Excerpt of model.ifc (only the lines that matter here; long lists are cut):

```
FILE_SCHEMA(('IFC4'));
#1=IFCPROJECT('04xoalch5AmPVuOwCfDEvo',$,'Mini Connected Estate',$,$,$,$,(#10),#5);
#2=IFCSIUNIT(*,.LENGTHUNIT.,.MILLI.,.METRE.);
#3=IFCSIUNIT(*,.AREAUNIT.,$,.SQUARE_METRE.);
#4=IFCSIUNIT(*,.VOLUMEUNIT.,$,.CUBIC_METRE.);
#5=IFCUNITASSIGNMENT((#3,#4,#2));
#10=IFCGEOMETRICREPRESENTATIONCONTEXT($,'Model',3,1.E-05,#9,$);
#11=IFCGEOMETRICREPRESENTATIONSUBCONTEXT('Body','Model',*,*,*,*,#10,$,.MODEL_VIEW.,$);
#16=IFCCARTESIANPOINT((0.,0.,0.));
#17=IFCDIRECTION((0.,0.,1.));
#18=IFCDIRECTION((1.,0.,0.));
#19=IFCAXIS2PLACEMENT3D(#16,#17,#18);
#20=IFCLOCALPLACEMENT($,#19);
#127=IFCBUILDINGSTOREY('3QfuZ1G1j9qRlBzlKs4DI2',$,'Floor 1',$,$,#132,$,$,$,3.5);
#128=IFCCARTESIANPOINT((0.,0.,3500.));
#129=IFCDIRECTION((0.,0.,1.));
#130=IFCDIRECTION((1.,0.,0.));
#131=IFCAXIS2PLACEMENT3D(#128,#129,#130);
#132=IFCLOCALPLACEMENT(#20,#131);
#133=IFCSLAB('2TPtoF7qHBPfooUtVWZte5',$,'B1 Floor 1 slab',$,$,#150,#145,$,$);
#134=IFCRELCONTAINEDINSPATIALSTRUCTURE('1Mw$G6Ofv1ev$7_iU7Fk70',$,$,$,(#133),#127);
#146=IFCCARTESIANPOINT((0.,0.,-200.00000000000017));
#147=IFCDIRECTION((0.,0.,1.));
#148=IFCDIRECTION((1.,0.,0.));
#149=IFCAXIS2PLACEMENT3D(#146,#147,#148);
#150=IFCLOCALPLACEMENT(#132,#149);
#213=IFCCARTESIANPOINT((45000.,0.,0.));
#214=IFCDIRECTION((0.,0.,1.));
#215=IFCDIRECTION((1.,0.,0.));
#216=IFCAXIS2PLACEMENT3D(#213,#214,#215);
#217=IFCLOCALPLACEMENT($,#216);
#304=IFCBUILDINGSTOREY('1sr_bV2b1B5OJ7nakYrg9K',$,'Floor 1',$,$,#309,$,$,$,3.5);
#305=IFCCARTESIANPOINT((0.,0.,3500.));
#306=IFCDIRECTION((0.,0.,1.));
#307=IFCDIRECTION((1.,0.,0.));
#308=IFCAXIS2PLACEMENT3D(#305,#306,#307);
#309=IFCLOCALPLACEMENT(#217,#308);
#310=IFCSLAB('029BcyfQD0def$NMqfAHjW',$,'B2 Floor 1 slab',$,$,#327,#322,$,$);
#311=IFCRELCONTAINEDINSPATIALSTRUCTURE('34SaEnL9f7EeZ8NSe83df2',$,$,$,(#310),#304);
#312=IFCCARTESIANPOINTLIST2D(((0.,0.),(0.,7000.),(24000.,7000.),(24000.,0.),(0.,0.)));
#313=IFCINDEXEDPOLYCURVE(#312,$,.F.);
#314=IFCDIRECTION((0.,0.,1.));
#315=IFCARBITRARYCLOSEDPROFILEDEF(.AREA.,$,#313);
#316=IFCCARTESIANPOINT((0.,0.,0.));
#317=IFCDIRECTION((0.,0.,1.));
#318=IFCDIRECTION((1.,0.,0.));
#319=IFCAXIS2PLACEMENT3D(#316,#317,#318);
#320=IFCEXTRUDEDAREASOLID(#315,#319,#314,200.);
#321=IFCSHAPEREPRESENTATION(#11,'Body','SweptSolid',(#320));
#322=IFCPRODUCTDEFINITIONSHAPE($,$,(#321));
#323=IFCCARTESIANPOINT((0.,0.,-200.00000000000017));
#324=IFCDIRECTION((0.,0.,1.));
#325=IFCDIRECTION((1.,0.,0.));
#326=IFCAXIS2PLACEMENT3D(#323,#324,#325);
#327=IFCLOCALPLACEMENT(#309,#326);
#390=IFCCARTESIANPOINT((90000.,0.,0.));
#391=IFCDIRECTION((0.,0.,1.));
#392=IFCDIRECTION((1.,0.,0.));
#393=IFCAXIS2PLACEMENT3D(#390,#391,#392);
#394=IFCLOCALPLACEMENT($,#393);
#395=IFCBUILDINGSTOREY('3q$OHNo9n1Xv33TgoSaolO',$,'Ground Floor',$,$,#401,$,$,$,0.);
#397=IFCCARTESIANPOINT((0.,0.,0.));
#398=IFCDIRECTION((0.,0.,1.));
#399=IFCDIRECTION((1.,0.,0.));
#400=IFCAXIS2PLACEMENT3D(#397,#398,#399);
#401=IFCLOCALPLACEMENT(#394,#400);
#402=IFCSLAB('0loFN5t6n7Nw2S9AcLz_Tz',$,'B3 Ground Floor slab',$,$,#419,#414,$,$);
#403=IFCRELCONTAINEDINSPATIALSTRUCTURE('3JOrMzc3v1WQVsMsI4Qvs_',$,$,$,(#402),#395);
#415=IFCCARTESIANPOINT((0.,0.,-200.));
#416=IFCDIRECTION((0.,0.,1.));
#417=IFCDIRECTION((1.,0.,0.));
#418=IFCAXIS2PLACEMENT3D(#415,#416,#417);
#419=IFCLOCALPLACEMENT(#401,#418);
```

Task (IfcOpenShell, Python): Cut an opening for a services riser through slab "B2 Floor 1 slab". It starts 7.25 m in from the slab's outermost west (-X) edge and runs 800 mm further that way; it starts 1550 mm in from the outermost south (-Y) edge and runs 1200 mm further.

```python
import numpy as np
import ifcopenshell
import ifcopenshell.api.feature
import ifcopenshell.api.geometry
import ifcopenshell.api.root
import ifcopenshell.geom
import ifcopenshell.util.placement
import ifcopenshell.util.representation
import ifcopenshell.util.shape
import ifcopenshell.util.unit

model = ifcopenshell.open("model.ifc")
unit_scale = ifcopenshell.util.unit.calculate_unit_scale(model)
settings = ifcopenshell.geom.settings()


def volume(element):
    """Net volume in cubic metres, openings subtracted."""
    shape = ifcopenshell.geom.create_shape(settings, element)
    return ifcopenshell.util.shape.get_volume(shape.geometry)


slab = model.by_id(310)
before = volume(slab)

# Extent in the slab's own axes, in metres. The edges named are its -X and -Y sides.
slab_shape = ifcopenshell.geom.create_shape(settings, slab)
vertices = ifcopenshell.util.shape.get_vertices(slab_shape.geometry)
x_min, y_min, bottom = vertices.min(axis=0)
top = vertices[:, 2].max()

opening = ifcopenshell.api.root.create_entity(model, ifc_class="IfcOpeningElement", name="Services riser opening", predefined_type="OPENING")
context = ifcopenshell.util.representation.get_context(model, "Model", "Body", "MODEL_VIEW")
width, depth = 0.8, 1.2
outline = [(0.0, 0.0), (width, 0.0), (width, depth), (0.0, depth), (0.0, 0.0)]
# Overshoot both faces by 50 mm so the cut is clean.
shape = ifcopenshell.api.geometry.add_slab_representation(
    model, context=context, depth=top - bottom + 0.1, polyline=outline
)
ifcopenshell.api.geometry.assign_representation(model, product=opening, representation=shape)

matrix = ifcopenshell.util.placement.get_local_placement(slab.ObjectPlacement)
matrix[:, 3] = matrix @ np.append(np.array([x_min + 7.25, y_min + 1.55, bottom - 0.05]) / unit_scale, 1.0)
ifcopenshell.api.geometry.edit_object_placement(model, product=opening, matrix=matrix, is_si=False)
ifcopenshell.api.feature.add_feature(model, feature=opening, element=slab)

after = volume(slab)

print(f"slab volume {before:.3f} -> {after:.3f} m3")

model.write("model_v2.ifc")
```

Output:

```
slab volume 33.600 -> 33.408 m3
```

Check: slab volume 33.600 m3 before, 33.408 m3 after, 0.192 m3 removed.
